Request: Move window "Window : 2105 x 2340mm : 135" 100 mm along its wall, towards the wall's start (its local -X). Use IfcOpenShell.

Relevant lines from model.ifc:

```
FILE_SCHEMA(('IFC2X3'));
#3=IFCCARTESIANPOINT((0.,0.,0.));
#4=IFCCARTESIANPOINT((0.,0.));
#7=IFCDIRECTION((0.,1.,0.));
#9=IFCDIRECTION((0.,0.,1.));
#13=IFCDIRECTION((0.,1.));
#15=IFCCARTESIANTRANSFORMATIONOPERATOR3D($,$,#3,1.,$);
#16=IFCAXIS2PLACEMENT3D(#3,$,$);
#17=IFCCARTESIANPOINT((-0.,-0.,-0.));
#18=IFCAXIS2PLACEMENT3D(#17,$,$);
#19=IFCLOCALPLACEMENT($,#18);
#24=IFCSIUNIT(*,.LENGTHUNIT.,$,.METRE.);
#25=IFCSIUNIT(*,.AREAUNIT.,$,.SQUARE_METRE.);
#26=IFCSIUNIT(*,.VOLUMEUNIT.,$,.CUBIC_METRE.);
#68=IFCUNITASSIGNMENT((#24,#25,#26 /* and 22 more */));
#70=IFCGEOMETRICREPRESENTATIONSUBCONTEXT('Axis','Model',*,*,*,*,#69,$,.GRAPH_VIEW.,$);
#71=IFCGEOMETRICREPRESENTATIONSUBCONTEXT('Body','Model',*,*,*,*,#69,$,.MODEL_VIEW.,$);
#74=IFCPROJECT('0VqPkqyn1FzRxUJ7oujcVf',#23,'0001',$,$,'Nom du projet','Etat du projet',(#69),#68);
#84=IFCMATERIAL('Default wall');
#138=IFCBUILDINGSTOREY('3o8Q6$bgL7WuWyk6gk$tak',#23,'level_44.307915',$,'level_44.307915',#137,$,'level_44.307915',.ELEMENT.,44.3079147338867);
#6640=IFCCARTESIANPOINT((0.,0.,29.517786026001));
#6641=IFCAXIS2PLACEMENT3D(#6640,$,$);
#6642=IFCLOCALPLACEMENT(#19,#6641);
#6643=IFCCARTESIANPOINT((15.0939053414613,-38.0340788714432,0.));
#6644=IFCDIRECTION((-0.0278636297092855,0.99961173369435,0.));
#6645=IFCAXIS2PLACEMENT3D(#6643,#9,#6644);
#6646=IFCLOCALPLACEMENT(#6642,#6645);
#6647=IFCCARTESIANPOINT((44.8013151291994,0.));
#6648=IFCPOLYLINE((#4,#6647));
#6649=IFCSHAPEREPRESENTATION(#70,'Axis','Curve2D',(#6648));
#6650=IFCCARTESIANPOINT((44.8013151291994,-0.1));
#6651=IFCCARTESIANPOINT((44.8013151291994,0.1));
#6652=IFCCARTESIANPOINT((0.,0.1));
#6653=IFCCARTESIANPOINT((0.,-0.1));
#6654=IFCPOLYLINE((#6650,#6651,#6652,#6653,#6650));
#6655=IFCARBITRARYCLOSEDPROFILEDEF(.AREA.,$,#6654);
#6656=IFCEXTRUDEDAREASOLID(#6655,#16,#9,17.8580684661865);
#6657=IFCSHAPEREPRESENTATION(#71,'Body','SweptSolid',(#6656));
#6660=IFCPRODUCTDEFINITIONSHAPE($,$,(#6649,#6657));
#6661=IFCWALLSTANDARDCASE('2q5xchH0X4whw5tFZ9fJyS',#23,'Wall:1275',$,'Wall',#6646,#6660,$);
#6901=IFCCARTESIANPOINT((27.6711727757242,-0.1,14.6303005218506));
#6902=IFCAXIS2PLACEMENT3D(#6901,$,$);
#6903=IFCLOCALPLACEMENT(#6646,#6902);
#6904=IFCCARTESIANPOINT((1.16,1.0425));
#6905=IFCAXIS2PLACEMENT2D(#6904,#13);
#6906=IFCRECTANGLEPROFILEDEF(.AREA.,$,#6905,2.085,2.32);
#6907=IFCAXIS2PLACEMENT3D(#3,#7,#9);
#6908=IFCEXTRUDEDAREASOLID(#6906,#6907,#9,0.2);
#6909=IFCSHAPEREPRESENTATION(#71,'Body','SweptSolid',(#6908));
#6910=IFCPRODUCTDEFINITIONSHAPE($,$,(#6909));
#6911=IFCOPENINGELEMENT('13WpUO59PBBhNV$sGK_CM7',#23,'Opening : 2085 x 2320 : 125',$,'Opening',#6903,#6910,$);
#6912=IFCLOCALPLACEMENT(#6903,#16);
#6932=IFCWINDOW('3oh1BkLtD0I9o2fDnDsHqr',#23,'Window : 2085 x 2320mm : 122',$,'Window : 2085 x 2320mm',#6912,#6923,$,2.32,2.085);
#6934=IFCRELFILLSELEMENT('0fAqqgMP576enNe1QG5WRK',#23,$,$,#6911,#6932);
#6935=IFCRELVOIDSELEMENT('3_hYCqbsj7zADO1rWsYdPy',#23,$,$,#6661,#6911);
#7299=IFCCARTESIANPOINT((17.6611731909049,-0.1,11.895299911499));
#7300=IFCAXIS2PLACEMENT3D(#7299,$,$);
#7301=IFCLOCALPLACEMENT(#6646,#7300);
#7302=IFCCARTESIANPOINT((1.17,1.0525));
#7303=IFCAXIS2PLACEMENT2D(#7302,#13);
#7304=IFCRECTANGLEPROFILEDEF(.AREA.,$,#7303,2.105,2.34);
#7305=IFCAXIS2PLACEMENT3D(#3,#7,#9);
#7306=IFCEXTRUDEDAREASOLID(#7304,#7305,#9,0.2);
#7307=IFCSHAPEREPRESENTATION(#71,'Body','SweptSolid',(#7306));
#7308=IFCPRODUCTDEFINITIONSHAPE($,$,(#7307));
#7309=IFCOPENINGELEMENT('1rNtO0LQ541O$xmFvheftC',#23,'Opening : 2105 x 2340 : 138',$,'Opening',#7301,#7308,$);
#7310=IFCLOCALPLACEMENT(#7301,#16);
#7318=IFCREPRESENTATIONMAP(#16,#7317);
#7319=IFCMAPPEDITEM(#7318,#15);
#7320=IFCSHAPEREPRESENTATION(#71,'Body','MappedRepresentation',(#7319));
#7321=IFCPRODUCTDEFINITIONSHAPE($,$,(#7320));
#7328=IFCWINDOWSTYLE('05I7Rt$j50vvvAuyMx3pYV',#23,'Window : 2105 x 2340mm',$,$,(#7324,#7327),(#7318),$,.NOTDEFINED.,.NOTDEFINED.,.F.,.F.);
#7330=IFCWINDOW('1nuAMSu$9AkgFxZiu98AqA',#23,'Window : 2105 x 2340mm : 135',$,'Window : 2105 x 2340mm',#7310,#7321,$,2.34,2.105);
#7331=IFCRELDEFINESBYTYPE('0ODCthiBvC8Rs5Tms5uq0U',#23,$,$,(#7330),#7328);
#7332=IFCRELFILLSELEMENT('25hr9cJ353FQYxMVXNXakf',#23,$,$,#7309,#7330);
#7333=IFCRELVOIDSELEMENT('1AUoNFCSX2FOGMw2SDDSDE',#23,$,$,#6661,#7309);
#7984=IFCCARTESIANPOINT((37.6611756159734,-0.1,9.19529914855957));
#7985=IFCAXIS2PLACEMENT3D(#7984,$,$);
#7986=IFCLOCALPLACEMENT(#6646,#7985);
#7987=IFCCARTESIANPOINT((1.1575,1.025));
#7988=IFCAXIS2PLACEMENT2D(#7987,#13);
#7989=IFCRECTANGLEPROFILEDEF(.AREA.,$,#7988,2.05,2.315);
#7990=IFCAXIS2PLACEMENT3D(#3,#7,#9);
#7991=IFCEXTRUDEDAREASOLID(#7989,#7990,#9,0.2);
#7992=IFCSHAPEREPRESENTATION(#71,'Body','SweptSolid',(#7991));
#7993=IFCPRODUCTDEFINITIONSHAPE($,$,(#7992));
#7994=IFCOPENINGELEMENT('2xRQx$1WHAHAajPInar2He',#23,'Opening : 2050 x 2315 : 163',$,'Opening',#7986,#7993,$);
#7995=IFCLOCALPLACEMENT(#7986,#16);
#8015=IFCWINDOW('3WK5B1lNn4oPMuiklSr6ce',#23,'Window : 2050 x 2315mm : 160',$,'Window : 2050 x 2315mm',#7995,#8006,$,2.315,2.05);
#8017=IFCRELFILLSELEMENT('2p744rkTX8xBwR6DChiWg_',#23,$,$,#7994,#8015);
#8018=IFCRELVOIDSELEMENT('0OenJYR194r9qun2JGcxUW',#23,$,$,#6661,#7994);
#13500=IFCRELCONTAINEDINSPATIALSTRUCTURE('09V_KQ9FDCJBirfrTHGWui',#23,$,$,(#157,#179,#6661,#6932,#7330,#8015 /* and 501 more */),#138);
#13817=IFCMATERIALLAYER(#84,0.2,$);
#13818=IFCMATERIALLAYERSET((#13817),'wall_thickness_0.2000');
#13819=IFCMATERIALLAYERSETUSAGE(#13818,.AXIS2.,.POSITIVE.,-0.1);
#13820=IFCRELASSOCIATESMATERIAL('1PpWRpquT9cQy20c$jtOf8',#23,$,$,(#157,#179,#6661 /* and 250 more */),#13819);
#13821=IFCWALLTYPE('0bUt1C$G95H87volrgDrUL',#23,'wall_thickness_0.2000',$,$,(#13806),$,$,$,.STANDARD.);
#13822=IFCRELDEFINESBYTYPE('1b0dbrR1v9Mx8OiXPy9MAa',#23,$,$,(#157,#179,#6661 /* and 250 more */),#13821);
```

```python
import ifcopenshell
import ifcopenshell.api.geometry
import ifcopenshell.util.placement

model = ifcopenshell.open("model.ifc")

window = model.by_guid("1nuAMSu$9AkgFxZiu98AqA")
opening = window.FillsVoids[0].RelatingOpeningElement
wall = opening.VoidsElements[0].RelatingBuildingElement

wall_matrix = ifcopenshell.util.placement.get_local_placement(wall.ObjectPlacement)
shift = wall_matrix[:3, 0] * -0.1
before = ifcopenshell.util.placement.get_local_placement(window.ObjectPlacement)[:3, 3].copy()

# The window is placed relative to its opening, so it follows when the opening moves.
matrix = ifcopenshell.util.placement.get_local_placement(opening.ObjectPlacement)
matrix[:3, 3] += shift
ifcopenshell.api.geometry.edit_object_placement(
    model, product=opening, matrix=matrix, is_si=False, should_transform_children=True
)

after = ifcopenshell.util.placement.get_local_placement(window.ObjectPlacement)[:3, 3]
print("window moved by", (after - before).round(3) + 0.0)

model.write("model_rev.ifc")
```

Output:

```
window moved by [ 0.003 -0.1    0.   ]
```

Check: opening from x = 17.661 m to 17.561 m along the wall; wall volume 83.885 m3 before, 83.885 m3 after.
